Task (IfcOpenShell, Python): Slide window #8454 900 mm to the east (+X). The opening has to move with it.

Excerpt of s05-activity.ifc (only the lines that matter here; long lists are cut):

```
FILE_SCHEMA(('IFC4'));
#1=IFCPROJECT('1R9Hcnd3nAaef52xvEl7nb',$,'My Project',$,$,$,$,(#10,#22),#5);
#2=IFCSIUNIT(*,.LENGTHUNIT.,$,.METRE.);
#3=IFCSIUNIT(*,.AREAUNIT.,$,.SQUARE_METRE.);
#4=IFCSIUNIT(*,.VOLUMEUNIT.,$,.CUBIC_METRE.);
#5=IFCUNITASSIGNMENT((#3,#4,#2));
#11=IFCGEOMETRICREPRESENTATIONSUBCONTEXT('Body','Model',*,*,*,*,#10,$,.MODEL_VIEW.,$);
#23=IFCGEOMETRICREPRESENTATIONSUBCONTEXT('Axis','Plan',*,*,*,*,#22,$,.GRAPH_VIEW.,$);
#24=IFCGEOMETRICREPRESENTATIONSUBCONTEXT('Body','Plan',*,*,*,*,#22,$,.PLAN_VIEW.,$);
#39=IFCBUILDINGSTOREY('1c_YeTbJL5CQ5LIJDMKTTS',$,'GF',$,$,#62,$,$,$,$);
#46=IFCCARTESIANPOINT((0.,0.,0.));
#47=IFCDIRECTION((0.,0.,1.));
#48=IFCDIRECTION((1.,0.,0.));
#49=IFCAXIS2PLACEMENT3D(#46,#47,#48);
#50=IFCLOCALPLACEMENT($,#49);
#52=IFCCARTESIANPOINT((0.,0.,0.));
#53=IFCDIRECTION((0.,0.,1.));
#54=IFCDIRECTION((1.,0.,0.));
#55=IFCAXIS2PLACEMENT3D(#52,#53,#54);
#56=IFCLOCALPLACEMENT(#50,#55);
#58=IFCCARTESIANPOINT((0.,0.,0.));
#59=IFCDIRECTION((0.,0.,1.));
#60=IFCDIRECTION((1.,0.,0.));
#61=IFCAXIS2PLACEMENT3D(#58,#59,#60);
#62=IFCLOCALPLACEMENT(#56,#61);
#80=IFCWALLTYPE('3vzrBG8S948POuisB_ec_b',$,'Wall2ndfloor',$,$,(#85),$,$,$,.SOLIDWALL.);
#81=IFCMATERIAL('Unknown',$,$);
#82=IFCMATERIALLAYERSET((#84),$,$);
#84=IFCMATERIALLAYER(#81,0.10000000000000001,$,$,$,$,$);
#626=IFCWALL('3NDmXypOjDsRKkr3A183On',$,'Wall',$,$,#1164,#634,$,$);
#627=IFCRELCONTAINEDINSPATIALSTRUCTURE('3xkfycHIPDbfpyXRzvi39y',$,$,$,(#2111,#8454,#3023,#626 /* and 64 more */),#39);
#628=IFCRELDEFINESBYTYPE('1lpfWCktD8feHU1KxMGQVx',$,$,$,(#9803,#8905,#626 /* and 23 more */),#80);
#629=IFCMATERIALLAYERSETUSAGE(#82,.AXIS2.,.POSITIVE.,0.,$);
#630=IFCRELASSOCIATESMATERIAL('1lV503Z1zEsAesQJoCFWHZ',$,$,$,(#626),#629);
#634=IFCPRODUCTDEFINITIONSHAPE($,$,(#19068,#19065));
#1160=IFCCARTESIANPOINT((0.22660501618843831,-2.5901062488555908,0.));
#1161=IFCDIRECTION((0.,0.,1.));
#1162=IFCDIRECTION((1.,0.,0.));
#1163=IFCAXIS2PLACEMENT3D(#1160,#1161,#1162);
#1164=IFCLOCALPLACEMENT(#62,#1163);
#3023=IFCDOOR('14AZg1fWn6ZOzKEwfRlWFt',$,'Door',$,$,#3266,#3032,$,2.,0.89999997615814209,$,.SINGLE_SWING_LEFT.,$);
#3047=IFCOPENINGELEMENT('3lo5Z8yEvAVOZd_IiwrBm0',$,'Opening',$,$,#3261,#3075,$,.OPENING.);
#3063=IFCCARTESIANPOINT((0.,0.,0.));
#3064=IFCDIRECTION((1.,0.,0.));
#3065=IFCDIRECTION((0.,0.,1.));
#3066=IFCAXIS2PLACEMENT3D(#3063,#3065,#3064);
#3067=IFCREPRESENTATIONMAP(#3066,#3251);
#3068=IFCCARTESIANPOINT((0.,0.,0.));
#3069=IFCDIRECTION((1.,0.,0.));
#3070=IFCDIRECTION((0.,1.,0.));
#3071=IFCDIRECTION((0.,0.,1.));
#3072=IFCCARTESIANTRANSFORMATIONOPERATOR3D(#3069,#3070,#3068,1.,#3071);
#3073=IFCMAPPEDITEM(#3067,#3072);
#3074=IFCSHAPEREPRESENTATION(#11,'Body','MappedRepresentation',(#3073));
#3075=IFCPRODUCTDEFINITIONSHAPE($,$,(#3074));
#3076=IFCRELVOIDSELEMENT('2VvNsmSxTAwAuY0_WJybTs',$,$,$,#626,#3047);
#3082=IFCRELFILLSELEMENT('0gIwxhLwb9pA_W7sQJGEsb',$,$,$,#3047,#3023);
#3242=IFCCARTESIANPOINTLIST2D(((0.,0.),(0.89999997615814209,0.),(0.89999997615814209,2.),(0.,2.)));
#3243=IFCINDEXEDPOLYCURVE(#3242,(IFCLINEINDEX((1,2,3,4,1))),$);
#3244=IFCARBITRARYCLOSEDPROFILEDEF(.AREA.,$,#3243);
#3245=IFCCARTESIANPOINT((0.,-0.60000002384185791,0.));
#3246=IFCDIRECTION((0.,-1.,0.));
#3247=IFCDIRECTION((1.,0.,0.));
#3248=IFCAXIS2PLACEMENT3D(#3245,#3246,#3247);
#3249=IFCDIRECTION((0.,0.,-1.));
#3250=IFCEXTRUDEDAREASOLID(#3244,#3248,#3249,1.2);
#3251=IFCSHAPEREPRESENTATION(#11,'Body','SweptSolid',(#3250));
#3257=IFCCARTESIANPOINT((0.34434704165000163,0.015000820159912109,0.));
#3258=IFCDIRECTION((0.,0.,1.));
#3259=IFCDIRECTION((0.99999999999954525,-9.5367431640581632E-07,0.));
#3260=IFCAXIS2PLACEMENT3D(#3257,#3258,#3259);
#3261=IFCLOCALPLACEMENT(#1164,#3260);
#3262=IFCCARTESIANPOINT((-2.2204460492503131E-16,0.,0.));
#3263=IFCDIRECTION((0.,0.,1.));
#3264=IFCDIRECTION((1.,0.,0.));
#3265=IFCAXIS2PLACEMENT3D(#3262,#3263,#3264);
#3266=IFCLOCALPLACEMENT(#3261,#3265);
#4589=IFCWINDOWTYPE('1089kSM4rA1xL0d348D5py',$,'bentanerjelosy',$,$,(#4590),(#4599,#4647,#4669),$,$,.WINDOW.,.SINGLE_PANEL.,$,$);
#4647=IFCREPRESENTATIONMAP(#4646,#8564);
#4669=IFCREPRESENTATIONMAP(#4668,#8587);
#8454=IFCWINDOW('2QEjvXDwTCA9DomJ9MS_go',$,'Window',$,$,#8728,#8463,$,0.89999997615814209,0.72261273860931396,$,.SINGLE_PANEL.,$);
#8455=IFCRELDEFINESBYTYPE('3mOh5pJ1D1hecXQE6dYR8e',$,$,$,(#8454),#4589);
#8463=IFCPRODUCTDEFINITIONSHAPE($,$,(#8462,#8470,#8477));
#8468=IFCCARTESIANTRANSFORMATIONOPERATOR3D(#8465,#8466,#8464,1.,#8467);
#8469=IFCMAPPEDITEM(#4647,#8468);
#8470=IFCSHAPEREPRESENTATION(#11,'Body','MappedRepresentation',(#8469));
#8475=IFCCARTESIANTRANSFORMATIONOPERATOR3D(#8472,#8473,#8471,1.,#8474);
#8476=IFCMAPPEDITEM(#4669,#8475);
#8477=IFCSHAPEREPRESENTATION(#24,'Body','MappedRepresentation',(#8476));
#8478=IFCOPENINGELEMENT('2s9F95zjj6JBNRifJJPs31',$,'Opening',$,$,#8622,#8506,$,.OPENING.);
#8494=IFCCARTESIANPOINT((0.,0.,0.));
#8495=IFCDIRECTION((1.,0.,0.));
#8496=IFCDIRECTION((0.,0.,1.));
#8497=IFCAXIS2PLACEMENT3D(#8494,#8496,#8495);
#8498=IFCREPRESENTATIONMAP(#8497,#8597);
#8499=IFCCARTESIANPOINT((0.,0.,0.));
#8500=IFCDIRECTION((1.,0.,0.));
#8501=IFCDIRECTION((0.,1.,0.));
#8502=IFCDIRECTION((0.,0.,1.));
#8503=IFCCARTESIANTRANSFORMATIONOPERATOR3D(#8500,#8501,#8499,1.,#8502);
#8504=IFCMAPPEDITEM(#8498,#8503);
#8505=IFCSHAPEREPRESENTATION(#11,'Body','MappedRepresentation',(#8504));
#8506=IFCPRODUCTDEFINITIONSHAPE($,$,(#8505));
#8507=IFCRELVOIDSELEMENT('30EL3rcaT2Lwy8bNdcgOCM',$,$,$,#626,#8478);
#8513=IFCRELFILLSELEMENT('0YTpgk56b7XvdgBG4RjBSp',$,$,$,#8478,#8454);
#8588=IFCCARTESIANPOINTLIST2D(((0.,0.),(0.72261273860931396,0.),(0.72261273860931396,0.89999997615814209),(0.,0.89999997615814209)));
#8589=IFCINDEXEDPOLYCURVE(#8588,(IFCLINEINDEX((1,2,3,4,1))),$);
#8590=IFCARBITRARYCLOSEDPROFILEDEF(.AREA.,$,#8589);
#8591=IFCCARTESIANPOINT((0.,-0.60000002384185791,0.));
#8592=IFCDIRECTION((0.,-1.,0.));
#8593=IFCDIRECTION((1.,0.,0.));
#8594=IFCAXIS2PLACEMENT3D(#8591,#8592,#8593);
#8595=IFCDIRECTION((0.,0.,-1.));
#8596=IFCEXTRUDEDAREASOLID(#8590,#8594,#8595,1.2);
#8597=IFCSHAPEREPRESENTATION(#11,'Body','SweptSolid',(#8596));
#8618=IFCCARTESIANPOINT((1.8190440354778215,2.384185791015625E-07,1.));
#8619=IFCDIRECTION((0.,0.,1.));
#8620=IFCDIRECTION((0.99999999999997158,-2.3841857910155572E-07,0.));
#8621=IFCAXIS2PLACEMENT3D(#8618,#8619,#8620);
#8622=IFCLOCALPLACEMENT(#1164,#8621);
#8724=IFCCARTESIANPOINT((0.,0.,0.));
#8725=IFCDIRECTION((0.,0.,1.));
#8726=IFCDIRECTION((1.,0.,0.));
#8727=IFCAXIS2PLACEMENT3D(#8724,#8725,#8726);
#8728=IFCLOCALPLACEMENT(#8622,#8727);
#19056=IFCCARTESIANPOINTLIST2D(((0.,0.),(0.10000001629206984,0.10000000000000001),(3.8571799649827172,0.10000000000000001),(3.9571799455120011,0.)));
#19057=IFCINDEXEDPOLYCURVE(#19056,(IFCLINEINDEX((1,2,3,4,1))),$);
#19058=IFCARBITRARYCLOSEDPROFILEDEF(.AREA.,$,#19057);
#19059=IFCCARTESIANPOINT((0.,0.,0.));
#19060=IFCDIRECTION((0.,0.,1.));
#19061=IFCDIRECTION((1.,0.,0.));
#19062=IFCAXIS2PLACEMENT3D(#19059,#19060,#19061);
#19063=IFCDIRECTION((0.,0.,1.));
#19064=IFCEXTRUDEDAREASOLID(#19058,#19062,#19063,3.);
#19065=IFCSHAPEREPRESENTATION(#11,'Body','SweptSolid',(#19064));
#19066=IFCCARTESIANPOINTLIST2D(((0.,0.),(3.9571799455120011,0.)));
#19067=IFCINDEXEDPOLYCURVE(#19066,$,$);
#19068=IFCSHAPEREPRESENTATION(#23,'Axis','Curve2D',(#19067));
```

```python
import ifcopenshell
import ifcopenshell.api.geometry
import ifcopenshell.util.placement
import ifcopenshell.util.unit

model = ifcopenshell.open("s05-activity.ifc")
unit_scale = ifcopenshell.util.unit.calculate_unit_scale(model)

window = model.by_guid("2QEjvXDwTCA9DomJ9MS_go")
opening = window.FillsVoids[0].RelatingOpeningElement
wall = opening.VoidsElements[0].RelatingBuildingElement

wall_matrix = ifcopenshell.util.placement.get_local_placement(wall.ObjectPlacement)
shift = wall_matrix[:3, 0] * 0.9 / unit_scale
before = ifcopenshell.util.placement.get_local_placement(window.ObjectPlacement)[:3, 3].copy()

# The window is placed relative to its opening, so it follows when the opening moves.
matrix = ifcopenshell.util.placement.get_local_placement(opening.ObjectPlacement)
matrix[:3, 3] += shift
ifcopenshell.api.geometry.edit_object_placement(
    model, product=opening, matrix=matrix, is_si=False, should_transform_children=True
)

after = ifcopenshell.util.placement.get_local_placement(window.ObjectPlacement)[:3, 3]
print("window moved by", (after - before).round(3) + 0.0)

model.write("s05-activity_updated.ifc")
```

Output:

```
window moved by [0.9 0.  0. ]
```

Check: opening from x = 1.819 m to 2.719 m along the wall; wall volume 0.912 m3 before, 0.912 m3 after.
